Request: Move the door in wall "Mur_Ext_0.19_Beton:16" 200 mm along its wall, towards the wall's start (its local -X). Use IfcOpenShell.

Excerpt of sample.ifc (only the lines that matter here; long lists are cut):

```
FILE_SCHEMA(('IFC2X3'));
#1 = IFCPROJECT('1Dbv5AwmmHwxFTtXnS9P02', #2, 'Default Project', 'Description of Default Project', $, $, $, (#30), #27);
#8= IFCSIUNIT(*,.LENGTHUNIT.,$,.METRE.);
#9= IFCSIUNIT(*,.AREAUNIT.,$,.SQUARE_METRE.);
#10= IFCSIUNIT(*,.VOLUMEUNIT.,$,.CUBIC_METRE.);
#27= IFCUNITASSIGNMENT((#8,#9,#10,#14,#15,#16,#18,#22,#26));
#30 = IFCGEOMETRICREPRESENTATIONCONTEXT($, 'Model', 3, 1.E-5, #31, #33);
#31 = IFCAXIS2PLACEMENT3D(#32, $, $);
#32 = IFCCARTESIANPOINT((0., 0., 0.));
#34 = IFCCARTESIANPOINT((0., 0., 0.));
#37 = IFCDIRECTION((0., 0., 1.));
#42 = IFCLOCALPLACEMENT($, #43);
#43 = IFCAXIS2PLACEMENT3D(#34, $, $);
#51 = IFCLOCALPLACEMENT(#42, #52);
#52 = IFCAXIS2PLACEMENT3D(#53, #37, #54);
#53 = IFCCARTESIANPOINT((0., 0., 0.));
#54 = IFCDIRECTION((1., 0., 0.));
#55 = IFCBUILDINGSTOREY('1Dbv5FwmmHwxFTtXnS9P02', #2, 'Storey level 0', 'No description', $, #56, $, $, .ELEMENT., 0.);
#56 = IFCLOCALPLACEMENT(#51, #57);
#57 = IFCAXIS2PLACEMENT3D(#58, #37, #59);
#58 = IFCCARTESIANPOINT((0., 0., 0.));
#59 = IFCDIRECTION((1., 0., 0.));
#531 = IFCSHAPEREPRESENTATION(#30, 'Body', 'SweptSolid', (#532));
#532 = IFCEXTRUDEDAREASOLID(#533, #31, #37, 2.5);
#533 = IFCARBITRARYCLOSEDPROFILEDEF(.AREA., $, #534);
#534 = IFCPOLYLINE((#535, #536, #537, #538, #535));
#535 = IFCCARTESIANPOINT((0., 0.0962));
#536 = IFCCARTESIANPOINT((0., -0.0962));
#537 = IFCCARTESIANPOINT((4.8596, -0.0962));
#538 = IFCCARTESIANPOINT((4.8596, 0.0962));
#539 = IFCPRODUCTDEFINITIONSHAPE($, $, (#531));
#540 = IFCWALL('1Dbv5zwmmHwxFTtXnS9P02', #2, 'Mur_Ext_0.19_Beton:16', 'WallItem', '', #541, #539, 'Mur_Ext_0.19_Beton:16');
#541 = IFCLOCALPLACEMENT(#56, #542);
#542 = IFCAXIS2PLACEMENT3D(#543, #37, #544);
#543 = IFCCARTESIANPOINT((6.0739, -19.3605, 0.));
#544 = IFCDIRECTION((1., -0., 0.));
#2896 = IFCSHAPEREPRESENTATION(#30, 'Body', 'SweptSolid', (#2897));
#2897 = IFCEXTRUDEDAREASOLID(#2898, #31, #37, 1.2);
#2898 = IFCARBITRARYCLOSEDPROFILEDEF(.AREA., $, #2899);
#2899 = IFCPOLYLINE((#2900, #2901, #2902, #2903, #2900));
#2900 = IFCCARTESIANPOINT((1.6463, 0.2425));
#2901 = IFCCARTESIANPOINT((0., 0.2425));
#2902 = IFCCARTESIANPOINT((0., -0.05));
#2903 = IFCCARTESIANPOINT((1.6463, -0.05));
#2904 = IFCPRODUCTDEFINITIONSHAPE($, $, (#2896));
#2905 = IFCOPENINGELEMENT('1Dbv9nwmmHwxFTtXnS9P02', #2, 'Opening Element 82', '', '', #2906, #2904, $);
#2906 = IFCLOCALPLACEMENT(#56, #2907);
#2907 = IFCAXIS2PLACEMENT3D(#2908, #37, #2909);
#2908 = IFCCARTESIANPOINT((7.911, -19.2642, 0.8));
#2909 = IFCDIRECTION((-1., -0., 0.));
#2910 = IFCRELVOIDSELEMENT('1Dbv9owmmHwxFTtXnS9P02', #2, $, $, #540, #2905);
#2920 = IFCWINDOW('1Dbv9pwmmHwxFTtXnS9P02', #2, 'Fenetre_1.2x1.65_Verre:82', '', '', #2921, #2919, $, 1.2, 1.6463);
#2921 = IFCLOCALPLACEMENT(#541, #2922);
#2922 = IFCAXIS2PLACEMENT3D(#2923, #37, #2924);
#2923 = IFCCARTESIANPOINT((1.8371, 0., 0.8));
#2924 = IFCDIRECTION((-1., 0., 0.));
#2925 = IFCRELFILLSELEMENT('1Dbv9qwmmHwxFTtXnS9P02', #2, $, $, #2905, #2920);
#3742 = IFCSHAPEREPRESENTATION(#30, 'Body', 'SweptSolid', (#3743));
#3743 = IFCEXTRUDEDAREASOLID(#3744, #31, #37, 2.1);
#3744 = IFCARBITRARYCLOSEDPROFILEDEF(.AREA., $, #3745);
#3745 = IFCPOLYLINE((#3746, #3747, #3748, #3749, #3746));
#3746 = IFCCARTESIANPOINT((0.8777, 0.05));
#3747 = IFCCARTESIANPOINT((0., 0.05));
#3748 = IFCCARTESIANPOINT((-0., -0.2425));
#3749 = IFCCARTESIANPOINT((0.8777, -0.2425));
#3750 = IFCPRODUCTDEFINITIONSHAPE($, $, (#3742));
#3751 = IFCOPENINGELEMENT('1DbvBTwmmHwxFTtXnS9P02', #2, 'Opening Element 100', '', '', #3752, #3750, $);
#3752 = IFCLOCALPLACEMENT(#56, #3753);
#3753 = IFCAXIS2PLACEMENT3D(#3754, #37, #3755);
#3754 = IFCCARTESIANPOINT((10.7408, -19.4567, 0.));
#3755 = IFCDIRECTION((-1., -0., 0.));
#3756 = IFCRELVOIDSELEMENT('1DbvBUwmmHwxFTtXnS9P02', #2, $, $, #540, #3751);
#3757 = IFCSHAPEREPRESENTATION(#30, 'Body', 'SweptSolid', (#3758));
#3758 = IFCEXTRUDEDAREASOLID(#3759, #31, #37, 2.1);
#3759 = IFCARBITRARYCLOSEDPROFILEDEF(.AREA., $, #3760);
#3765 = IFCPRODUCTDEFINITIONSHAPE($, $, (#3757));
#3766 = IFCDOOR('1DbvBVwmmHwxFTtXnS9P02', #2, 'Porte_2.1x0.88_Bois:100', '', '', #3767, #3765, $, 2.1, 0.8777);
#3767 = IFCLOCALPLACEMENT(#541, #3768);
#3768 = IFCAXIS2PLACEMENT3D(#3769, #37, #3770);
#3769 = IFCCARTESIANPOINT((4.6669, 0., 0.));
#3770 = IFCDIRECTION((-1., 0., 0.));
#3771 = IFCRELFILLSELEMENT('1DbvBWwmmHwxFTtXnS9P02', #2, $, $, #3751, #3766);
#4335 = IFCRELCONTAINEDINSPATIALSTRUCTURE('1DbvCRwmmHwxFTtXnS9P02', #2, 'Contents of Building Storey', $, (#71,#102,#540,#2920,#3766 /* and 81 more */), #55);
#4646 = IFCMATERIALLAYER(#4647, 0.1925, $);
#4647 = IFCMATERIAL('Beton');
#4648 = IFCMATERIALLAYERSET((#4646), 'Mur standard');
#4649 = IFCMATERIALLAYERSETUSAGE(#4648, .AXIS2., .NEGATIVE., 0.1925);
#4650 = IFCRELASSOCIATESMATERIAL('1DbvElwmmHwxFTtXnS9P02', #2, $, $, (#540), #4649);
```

```python
import ifcopenshell
import ifcopenshell.api.geometry
import ifcopenshell.util.placement

model = ifcopenshell.open("sample.ifc")

door = model.by_id(3766)
opening = door.FillsVoids[0].RelatingOpeningElement
wall = opening.VoidsElements[0].RelatingBuildingElement

wall_matrix = ifcopenshell.util.placement.get_local_placement(wall.ObjectPlacement)
shift = wall_matrix[:3, 0] * -0.2
before = ifcopenshell.util.placement.get_local_placement(door.ObjectPlacement)[:3, 3].copy()

# The door is not placed relative to its opening, so move both.
for product in (opening, door):
    matrix = ifcopenshell.util.placement.get_local_placement(product.ObjectPlacement)
    matrix[:3, 3] += shift
    ifcopenshell.api.geometry.edit_object_placement(model, product=product, matrix=matrix, is_si=False)

after = ifcopenshell.util.placement.get_local_placement(door.ObjectPlacement)[:3, 3]
print("door moved by", (after - before).round(3) + 0.0)

model.write("sample_edited.ifc")
```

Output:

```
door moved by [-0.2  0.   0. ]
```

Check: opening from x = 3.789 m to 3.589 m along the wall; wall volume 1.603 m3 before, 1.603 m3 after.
